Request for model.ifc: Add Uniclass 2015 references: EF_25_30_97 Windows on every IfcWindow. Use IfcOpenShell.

First a look at what the model holds.

```python
import ifcopenshell

model = ifcopenshell.open("model.ifc")
print(model.schema)
print("classifications:", [c.Name for c in model.by_type("IfcClassification")])
for ifc_class in ("IfcDoor", "IfcRoof", "IfcStair", "IfcWall", "IfcWindow"):
    print(ifc_class, len(model.by_type(ifc_class)))
```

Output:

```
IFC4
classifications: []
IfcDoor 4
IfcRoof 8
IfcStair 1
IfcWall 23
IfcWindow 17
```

```python
import ifcopenshell
import ifcopenshell.api.classification

model = ifcopenshell.open("model.ifc")

system = ifcopenshell.api.classification.add_classification(model, classification="Uniclass 2015")

codes = {
    "IfcWindow": ("EF_25_30_97", "Windows"),
}
for ifc_class, (code, name) in codes.items():
    products = model.by_type(ifc_class)
    ifcopenshell.api.classification.add_reference(
        model, products=products, classification=system, identification=code, name=name
    )
    print(code, len(products))

model.write("model_edited.ifc")
```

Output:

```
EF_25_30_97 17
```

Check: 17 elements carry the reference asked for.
